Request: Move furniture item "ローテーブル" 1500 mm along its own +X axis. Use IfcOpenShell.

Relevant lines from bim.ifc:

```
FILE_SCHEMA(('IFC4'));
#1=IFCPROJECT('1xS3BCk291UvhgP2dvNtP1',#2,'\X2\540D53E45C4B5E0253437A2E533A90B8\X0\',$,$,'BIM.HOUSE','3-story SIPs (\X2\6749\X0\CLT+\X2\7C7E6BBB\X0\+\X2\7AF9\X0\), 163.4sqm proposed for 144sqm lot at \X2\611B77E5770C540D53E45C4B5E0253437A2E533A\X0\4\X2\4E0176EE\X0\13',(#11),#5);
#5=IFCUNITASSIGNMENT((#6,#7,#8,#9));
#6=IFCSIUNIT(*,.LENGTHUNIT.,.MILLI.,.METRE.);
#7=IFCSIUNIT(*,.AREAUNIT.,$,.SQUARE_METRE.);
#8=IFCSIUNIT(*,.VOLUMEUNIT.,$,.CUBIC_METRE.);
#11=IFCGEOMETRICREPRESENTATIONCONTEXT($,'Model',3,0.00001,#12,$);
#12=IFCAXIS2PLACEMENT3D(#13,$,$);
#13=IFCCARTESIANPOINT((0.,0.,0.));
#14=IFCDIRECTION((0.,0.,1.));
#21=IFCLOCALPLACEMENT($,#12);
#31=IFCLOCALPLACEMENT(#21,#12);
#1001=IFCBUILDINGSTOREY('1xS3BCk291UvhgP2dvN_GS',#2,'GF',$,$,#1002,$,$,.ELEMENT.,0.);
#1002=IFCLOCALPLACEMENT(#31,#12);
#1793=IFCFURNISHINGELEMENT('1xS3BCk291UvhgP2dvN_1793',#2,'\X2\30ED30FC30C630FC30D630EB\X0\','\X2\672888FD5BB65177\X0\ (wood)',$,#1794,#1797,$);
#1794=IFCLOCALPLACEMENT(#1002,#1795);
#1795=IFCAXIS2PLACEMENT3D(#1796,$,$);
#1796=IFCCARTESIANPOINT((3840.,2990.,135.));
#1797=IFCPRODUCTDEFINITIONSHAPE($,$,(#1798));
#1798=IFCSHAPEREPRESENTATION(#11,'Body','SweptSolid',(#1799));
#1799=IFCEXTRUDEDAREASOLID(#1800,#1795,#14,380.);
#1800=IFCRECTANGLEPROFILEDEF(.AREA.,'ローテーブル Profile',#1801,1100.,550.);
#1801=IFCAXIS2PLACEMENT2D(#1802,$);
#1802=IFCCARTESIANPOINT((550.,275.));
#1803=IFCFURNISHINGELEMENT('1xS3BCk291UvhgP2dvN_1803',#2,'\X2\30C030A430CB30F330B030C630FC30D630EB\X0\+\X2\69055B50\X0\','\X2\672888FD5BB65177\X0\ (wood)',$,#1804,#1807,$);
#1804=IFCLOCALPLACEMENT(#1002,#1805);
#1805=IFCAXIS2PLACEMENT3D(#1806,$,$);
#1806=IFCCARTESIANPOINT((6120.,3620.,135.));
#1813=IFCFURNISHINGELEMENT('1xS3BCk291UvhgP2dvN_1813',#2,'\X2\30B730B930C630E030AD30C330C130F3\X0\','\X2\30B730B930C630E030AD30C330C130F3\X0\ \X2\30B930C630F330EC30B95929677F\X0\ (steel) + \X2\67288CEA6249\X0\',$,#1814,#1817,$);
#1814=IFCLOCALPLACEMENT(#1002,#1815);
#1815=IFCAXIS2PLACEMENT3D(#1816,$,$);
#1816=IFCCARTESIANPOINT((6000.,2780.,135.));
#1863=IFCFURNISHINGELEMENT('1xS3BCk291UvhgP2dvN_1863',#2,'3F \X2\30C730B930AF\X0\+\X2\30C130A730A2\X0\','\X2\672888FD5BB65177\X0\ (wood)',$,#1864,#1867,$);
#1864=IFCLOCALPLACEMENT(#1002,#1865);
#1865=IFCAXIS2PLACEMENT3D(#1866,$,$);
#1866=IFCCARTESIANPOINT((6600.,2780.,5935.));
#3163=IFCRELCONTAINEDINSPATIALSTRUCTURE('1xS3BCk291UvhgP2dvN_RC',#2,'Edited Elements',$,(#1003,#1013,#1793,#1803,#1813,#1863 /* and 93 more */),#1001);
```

```python
import ifcopenshell
import ifcopenshell.api.geometry
import ifcopenshell.util.placement

model = ifcopenshell.open("bim.ifc")

item = model.by_guid("1xS3BCk291UvhgP2dvN_1793")
matrix = ifcopenshell.util.placement.get_local_placement(item.ObjectPlacement)
matrix[:3, 3] += matrix[:3, 0] * 1500.0
ifcopenshell.api.geometry.edit_object_placement(model, product=item, matrix=matrix, is_si=False)

print(ifcopenshell.util.placement.get_local_placement(item.ObjectPlacement).round(3) + 0.0)

model.write("bim_edited.ifc")
```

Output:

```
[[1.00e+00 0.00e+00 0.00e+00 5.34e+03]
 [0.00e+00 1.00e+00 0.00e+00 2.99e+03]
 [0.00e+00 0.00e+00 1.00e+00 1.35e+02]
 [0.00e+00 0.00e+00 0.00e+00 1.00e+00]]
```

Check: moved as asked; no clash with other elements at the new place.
